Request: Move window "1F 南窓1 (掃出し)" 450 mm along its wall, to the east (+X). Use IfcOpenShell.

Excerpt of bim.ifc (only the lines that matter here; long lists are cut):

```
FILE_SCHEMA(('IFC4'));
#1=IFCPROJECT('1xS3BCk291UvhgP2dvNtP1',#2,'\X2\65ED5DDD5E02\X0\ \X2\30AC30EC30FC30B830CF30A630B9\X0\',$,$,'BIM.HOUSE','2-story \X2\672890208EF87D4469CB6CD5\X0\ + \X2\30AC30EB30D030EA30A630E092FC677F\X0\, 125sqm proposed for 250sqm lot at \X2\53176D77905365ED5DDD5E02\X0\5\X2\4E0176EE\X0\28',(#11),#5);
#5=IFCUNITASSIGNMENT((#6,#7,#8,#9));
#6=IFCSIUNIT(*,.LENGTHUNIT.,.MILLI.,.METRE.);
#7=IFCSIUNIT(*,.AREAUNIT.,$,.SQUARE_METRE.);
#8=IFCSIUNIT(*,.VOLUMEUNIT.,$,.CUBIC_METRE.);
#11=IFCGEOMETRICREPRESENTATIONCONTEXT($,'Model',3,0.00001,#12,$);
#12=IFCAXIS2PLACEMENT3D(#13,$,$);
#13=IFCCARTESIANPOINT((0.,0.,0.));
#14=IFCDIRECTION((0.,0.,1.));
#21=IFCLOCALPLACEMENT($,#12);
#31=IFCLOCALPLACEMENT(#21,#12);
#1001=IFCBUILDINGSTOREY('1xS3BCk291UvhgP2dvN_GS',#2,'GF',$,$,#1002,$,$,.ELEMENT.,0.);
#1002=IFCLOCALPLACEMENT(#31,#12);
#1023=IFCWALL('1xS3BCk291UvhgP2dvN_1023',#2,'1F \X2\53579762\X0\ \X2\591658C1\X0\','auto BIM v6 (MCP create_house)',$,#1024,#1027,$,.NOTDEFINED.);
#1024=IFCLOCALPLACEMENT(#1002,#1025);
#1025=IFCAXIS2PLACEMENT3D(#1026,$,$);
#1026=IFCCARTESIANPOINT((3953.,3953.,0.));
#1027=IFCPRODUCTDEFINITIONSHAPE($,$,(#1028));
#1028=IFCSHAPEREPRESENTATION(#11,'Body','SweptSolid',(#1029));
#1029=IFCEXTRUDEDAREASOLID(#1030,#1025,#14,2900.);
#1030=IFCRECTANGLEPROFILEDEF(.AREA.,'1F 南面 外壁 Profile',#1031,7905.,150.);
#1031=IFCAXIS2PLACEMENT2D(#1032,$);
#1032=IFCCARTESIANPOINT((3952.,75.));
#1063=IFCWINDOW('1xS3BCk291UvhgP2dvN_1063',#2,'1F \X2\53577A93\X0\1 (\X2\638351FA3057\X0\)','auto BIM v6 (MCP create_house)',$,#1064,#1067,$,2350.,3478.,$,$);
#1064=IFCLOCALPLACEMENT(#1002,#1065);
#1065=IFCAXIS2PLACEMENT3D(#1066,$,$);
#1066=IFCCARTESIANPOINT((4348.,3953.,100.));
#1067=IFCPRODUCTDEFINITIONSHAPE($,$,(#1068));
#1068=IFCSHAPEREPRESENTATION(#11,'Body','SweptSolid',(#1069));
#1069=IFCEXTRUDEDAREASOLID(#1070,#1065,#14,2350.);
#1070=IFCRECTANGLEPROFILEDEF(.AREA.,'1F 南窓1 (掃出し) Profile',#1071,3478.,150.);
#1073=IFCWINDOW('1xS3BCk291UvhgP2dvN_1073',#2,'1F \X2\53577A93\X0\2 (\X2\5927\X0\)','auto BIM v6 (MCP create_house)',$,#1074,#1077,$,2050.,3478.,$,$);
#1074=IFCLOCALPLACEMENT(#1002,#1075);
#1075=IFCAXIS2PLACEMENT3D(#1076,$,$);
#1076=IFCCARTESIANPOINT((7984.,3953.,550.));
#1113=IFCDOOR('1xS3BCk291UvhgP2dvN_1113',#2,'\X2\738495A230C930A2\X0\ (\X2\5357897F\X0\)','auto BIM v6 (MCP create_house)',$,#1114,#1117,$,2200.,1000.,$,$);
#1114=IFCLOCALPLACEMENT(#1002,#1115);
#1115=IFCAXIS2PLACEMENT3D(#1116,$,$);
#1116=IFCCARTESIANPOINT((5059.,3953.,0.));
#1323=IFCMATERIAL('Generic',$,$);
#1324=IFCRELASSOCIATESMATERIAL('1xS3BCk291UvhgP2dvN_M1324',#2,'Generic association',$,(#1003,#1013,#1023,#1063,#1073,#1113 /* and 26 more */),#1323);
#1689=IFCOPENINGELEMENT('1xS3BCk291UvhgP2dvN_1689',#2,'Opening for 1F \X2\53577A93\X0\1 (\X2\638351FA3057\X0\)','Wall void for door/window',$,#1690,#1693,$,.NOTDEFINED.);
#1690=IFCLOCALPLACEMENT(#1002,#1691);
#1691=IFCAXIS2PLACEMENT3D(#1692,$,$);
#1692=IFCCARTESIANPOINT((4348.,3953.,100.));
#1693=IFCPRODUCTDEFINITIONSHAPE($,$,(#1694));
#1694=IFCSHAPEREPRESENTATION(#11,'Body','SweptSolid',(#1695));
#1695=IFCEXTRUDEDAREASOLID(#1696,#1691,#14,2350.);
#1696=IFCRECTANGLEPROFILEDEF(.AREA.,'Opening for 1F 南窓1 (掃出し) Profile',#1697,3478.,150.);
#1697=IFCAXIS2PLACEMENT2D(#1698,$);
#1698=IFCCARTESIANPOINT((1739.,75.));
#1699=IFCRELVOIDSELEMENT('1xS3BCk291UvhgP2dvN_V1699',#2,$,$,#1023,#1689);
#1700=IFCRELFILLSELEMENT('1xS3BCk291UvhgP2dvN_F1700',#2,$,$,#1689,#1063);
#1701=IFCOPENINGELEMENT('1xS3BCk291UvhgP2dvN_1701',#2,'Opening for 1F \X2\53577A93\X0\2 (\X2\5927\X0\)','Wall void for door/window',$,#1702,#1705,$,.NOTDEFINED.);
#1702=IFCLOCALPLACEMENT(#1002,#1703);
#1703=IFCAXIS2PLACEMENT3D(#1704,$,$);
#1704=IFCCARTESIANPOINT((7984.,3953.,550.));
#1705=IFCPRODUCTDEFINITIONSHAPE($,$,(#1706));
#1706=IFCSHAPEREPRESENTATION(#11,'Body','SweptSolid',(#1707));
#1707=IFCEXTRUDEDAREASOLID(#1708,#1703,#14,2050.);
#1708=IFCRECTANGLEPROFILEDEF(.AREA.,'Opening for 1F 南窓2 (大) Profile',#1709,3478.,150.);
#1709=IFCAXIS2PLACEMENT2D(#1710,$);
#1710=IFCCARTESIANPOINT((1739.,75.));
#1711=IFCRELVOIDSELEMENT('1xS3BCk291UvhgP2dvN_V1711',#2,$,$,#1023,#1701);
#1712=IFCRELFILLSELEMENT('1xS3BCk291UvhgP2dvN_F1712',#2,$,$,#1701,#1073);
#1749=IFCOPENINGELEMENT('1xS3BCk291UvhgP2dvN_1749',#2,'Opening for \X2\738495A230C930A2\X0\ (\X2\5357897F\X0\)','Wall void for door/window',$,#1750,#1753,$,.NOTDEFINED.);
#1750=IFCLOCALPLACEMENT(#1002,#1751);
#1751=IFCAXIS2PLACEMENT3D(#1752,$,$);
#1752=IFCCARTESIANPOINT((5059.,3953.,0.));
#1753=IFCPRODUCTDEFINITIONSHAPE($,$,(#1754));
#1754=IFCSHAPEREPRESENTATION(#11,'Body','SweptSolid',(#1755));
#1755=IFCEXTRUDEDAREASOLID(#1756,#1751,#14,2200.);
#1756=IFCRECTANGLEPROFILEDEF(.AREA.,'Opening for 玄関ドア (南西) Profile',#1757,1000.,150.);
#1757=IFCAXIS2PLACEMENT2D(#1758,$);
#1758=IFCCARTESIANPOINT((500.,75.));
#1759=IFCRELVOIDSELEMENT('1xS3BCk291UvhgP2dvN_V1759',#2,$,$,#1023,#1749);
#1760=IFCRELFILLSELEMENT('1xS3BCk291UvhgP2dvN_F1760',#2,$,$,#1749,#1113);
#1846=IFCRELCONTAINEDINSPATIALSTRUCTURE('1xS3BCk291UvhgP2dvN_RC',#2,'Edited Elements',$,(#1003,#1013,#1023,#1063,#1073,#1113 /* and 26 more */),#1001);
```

```python
import ifcopenshell
import ifcopenshell.api.geometry
import ifcopenshell.util.placement

model = ifcopenshell.open("bim.ifc")

window = model.by_id(1063)
opening = window.FillsVoids[0].RelatingOpeningElement
wall = opening.VoidsElements[0].RelatingBuildingElement

wall_matrix = ifcopenshell.util.placement.get_local_placement(wall.ObjectPlacement)
shift = wall_matrix[:3, 0] * 450.0
before = ifcopenshell.util.placement.get_local_placement(window.ObjectPlacement)[:3, 3].copy()

# The window is not placed relative to its opening, so move both.
for product in (opening, window):
    matrix = ifcopenshell.util.placement.get_local_placement(product.ObjectPlacement)
    matrix[:3, 3] += shift
    ifcopenshell.api.geometry.edit_object_placement(model, product=product, matrix=matrix, is_si=False)

after = ifcopenshell.util.placement.get_local_placement(window.ObjectPlacement)[:3, 3]
print("window moved by", (after - before).round(3) + 0.0)

model.write("bim_edited.ifc")
```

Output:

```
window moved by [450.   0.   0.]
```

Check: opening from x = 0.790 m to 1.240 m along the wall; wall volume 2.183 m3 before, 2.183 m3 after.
